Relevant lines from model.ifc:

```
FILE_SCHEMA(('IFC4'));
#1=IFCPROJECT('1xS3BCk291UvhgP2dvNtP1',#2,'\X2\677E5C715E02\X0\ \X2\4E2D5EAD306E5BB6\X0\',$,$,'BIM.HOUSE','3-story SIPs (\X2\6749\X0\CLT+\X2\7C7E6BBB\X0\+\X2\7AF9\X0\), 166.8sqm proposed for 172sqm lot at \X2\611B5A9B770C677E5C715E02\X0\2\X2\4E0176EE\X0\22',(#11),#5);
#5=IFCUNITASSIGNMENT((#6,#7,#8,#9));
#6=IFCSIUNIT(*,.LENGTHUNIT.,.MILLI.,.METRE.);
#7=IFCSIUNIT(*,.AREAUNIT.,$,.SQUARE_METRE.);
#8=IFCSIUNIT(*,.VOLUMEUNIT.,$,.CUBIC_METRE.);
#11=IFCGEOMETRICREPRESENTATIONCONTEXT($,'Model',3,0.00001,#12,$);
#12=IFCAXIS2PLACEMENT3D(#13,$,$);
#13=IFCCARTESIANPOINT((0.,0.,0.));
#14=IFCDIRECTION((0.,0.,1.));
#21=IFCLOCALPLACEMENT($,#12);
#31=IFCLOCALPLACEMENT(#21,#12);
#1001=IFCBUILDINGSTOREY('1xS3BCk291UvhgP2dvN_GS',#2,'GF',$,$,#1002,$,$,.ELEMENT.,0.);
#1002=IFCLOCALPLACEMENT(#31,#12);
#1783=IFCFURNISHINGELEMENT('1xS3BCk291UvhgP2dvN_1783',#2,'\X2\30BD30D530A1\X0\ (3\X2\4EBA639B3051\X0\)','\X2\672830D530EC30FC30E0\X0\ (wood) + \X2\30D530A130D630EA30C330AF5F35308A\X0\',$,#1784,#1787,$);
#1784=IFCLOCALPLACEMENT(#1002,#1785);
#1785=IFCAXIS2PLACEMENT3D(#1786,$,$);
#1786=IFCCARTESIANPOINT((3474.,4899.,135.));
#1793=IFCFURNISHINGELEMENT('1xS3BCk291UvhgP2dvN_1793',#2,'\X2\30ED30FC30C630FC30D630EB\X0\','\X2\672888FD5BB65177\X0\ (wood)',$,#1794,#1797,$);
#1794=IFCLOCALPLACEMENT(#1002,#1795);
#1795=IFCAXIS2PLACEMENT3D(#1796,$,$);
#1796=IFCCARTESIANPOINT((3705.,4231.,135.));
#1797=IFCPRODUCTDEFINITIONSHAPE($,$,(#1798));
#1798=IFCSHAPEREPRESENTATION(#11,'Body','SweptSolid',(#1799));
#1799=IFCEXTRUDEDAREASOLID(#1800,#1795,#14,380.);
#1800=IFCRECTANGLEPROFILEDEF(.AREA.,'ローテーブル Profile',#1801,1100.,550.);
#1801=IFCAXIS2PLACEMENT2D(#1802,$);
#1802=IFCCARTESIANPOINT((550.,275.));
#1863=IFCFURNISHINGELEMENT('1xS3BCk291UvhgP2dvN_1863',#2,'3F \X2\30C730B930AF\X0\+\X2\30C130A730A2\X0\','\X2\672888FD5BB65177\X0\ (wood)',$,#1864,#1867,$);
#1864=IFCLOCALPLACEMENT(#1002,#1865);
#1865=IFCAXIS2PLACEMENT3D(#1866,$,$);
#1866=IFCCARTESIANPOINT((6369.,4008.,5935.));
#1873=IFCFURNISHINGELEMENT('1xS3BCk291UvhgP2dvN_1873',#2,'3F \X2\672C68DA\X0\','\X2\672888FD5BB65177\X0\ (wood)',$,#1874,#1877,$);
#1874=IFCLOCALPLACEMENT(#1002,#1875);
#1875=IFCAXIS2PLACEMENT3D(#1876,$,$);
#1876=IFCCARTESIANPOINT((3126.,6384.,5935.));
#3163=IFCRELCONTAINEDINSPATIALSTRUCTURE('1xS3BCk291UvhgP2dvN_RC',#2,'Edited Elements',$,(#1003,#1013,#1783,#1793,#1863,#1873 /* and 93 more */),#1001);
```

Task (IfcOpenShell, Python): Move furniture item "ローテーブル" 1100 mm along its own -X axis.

```python
import ifcopenshell
import ifcopenshell.api.geometry
import ifcopenshell.util.placement

model = ifcopenshell.open("model.ifc")

item = model.by_guid("1xS3BCk291UvhgP2dvN_1793")
matrix = ifcopenshell.util.placement.get_local_placement(item.ObjectPlacement)
matrix[:3, 3] -= matrix[:3, 0] * 1100.0
ifcopenshell.api.geometry.edit_object_placement(model, product=item, matrix=matrix, is_si=False)

print(ifcopenshell.util.placement.get_local_placement(item.ObjectPlacement).round(3) + 0.0)

model.write("model_rev.ifc")
```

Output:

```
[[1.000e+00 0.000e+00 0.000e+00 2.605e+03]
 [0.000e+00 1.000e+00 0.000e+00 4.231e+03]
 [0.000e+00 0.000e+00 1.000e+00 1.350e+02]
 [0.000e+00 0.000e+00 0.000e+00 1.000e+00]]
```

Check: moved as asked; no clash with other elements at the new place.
